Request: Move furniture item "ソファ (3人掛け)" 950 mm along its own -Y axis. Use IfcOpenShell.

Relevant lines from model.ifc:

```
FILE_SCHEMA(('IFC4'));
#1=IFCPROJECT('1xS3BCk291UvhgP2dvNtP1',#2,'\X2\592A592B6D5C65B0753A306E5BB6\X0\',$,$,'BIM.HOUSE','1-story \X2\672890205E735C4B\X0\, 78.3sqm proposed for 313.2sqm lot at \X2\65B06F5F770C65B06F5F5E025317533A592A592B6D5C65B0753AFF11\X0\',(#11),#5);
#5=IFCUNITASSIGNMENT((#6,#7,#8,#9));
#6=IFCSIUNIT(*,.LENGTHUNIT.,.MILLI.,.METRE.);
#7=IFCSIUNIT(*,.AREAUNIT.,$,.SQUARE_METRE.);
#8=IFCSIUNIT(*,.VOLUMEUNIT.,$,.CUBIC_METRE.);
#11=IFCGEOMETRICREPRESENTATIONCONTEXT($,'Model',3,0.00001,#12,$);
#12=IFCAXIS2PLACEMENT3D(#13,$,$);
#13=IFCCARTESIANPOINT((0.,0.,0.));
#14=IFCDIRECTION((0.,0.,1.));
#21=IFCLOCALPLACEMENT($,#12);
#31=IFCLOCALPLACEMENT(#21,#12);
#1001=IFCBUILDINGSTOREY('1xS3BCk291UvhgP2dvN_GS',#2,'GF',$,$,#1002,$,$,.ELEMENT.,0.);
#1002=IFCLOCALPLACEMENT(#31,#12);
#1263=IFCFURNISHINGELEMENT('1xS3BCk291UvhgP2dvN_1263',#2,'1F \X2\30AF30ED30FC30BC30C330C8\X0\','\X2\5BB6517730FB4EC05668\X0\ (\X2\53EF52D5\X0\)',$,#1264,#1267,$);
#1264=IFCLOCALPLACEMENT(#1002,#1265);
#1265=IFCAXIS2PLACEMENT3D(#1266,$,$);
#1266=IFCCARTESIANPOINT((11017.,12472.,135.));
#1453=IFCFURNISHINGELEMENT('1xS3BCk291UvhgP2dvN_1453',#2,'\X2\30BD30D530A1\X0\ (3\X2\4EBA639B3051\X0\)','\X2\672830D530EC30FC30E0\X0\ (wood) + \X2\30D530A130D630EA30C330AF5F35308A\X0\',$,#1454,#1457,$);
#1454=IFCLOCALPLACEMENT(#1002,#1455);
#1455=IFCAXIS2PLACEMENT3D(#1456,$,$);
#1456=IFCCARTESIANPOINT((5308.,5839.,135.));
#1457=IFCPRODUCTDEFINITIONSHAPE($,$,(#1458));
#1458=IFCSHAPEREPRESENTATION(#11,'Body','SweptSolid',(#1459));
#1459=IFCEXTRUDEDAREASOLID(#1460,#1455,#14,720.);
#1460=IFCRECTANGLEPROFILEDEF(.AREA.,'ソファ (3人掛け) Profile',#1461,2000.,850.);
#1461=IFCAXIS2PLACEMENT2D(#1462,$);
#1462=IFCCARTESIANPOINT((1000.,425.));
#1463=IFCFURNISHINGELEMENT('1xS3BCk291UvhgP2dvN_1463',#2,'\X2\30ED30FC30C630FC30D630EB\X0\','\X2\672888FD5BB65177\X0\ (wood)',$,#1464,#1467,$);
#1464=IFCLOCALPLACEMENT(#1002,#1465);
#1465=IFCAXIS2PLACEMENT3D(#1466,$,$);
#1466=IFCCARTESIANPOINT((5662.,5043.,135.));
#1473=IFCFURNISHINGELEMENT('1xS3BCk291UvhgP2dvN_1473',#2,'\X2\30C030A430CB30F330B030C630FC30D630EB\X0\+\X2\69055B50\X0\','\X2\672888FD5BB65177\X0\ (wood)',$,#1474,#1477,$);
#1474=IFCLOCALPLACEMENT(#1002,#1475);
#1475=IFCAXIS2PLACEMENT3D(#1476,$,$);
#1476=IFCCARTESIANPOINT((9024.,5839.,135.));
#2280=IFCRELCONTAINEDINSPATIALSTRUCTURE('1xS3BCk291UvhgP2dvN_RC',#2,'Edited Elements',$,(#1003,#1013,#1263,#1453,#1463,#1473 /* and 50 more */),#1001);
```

```python
import ifcopenshell
import ifcopenshell.api.geometry
import ifcopenshell.util.placement
import ifcopenshell.util.unit

model = ifcopenshell.open("model.ifc")
unit_scale = ifcopenshell.util.unit.calculate_unit_scale(model)

item = model.by_guid("1xS3BCk291UvhgP2dvN_1453")
matrix = ifcopenshell.util.placement.get_local_placement(item.ObjectPlacement)
matrix[:3, 3] -= matrix[:3, 1] * 0.95 / unit_scale
ifcopenshell.api.geometry.edit_object_placement(model, product=item, matrix=matrix, is_si=False)

print(ifcopenshell.util.placement.get_local_placement(item.ObjectPlacement).round(3) + 0.0)

model.write("model_rev.ifc")
```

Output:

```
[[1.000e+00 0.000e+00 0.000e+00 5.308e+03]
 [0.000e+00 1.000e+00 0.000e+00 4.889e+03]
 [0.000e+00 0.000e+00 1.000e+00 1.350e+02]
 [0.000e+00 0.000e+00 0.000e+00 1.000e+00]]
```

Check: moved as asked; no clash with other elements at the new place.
